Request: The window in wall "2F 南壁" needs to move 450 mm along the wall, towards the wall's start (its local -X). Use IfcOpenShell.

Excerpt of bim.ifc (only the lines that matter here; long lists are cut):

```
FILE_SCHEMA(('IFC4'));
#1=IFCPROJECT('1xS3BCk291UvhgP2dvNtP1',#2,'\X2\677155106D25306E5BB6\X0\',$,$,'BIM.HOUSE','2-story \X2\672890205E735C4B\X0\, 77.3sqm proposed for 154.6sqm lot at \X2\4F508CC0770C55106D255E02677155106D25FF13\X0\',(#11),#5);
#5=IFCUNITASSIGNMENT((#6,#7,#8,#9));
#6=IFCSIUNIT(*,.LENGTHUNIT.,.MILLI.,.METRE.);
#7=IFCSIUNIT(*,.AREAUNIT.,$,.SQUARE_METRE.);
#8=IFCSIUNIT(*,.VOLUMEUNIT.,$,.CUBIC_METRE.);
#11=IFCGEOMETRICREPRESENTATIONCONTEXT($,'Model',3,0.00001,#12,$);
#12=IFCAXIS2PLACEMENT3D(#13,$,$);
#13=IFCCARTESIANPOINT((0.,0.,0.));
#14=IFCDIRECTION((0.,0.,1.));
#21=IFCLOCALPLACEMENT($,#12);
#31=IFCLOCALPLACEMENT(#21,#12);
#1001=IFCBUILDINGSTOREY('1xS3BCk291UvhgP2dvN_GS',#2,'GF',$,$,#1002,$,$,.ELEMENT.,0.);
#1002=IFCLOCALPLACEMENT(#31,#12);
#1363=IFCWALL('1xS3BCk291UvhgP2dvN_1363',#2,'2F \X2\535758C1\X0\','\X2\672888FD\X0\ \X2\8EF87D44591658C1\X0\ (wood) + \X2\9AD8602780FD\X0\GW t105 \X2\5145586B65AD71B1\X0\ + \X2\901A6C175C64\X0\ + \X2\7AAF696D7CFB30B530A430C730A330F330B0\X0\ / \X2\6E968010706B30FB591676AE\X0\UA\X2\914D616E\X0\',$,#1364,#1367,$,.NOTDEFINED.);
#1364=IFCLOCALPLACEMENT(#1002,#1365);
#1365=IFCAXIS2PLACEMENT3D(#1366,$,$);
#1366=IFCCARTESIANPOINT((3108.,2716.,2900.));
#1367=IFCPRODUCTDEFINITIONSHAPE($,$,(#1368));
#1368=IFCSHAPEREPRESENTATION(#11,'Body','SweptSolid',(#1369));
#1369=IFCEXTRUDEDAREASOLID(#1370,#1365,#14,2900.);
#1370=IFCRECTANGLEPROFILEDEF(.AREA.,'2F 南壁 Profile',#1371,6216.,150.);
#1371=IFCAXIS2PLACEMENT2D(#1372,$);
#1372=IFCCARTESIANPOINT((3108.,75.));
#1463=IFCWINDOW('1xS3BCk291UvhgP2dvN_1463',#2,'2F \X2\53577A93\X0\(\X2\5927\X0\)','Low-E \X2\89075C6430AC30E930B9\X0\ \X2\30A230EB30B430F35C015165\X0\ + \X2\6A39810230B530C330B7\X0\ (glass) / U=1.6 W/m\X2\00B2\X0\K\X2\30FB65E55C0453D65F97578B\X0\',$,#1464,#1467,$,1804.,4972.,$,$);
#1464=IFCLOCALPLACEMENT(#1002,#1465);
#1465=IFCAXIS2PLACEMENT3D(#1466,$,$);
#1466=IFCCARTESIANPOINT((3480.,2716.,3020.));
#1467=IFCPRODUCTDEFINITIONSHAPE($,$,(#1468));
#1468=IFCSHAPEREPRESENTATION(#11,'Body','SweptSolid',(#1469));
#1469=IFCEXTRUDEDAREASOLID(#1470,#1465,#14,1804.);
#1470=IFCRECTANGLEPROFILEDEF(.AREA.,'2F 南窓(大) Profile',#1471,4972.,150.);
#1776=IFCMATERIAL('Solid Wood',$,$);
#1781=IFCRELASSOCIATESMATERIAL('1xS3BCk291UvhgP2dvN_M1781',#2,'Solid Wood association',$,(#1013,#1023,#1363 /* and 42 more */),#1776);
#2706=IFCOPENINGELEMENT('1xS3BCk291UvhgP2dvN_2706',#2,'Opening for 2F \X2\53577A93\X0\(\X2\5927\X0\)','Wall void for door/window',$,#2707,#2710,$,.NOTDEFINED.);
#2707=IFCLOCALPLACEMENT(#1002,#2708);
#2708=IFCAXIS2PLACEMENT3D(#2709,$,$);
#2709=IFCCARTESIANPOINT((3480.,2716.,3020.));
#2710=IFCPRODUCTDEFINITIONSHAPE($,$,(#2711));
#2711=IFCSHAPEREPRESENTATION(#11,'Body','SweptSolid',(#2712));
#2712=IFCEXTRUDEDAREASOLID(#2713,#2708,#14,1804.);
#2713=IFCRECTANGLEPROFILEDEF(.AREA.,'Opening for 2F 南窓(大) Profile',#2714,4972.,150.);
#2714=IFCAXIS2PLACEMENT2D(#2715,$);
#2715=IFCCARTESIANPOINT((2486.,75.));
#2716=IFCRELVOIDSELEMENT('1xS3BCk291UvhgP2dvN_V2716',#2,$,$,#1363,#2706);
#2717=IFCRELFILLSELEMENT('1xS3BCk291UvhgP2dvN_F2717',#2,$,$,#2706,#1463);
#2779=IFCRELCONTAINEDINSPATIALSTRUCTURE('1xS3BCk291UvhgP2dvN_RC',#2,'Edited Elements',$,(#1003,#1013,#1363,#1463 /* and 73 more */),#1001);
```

```python
import ifcopenshell
import ifcopenshell.api.geometry
import ifcopenshell.util.placement
import ifcopenshell.util.unit

model = ifcopenshell.open("bim.ifc")
unit_scale = ifcopenshell.util.unit.calculate_unit_scale(model)

window = model.by_guid("1xS3BCk291UvhgP2dvN_1463")
opening = window.FillsVoids[0].RelatingOpeningElement
wall = opening.VoidsElements[0].RelatingBuildingElement

wall_matrix = ifcopenshell.util.placement.get_local_placement(wall.ObjectPlacement)
shift = wall_matrix[:3, 0] * -0.45 / unit_scale
before = ifcopenshell.util.placement.get_local_placement(window.ObjectPlacement)[:3, 3].copy()

# The window is not placed relative to its opening, so move both.
for product in (opening, window):
    matrix = ifcopenshell.util.placement.get_local_placement(product.ObjectPlacement)
    matrix[:3, 3] += shift
    ifcopenshell.api.geometry.edit_object_placement(model, product=product, matrix=matrix, is_si=False)

after = ifcopenshell.util.placement.get_local_placement(window.ObjectPlacement)[:3, 3]
print("window moved by", (after - before).round(3) + 0.0)

model.write("bim_updated.ifc")
```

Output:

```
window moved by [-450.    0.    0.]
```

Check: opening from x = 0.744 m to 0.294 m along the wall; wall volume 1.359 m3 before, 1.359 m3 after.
